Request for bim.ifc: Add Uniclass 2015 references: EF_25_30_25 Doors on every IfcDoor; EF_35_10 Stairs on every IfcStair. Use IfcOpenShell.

First a look at what the model holds.

```python
import ifcopenshell

model = ifcopenshell.open("bim.ifc")
print(model.schema)
print("classifications:", [c.Name for c in model.by_type("IfcClassification")])
for ifc_class in ("IfcDoor", "IfcRoof", "IfcStair", "IfcWall", "IfcWindow"):
    print(ifc_class, len(model.by_type(ifc_class)))
```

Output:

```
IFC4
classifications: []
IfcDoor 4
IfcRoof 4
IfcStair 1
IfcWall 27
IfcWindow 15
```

```python
import ifcopenshell
import ifcopenshell.api.classification

model = ifcopenshell.open("bim.ifc")

system = ifcopenshell.api.classification.add_classification(model, classification="Uniclass 2015")

codes = {
    "IfcDoor": ("EF_25_30_25", "Doors"),
    "IfcStair": ("EF_35_10", "Stairs"),
}
for ifc_class, (code, name) in codes.items():
    products = model.by_type(ifc_class)
    ifcopenshell.api.classification.add_reference(
        model, products=products, classification=system, identification=code, name=name
    )
    print(code, len(products))

model.write("bim_updated.ifc")
```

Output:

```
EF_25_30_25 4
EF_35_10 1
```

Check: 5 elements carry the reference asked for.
